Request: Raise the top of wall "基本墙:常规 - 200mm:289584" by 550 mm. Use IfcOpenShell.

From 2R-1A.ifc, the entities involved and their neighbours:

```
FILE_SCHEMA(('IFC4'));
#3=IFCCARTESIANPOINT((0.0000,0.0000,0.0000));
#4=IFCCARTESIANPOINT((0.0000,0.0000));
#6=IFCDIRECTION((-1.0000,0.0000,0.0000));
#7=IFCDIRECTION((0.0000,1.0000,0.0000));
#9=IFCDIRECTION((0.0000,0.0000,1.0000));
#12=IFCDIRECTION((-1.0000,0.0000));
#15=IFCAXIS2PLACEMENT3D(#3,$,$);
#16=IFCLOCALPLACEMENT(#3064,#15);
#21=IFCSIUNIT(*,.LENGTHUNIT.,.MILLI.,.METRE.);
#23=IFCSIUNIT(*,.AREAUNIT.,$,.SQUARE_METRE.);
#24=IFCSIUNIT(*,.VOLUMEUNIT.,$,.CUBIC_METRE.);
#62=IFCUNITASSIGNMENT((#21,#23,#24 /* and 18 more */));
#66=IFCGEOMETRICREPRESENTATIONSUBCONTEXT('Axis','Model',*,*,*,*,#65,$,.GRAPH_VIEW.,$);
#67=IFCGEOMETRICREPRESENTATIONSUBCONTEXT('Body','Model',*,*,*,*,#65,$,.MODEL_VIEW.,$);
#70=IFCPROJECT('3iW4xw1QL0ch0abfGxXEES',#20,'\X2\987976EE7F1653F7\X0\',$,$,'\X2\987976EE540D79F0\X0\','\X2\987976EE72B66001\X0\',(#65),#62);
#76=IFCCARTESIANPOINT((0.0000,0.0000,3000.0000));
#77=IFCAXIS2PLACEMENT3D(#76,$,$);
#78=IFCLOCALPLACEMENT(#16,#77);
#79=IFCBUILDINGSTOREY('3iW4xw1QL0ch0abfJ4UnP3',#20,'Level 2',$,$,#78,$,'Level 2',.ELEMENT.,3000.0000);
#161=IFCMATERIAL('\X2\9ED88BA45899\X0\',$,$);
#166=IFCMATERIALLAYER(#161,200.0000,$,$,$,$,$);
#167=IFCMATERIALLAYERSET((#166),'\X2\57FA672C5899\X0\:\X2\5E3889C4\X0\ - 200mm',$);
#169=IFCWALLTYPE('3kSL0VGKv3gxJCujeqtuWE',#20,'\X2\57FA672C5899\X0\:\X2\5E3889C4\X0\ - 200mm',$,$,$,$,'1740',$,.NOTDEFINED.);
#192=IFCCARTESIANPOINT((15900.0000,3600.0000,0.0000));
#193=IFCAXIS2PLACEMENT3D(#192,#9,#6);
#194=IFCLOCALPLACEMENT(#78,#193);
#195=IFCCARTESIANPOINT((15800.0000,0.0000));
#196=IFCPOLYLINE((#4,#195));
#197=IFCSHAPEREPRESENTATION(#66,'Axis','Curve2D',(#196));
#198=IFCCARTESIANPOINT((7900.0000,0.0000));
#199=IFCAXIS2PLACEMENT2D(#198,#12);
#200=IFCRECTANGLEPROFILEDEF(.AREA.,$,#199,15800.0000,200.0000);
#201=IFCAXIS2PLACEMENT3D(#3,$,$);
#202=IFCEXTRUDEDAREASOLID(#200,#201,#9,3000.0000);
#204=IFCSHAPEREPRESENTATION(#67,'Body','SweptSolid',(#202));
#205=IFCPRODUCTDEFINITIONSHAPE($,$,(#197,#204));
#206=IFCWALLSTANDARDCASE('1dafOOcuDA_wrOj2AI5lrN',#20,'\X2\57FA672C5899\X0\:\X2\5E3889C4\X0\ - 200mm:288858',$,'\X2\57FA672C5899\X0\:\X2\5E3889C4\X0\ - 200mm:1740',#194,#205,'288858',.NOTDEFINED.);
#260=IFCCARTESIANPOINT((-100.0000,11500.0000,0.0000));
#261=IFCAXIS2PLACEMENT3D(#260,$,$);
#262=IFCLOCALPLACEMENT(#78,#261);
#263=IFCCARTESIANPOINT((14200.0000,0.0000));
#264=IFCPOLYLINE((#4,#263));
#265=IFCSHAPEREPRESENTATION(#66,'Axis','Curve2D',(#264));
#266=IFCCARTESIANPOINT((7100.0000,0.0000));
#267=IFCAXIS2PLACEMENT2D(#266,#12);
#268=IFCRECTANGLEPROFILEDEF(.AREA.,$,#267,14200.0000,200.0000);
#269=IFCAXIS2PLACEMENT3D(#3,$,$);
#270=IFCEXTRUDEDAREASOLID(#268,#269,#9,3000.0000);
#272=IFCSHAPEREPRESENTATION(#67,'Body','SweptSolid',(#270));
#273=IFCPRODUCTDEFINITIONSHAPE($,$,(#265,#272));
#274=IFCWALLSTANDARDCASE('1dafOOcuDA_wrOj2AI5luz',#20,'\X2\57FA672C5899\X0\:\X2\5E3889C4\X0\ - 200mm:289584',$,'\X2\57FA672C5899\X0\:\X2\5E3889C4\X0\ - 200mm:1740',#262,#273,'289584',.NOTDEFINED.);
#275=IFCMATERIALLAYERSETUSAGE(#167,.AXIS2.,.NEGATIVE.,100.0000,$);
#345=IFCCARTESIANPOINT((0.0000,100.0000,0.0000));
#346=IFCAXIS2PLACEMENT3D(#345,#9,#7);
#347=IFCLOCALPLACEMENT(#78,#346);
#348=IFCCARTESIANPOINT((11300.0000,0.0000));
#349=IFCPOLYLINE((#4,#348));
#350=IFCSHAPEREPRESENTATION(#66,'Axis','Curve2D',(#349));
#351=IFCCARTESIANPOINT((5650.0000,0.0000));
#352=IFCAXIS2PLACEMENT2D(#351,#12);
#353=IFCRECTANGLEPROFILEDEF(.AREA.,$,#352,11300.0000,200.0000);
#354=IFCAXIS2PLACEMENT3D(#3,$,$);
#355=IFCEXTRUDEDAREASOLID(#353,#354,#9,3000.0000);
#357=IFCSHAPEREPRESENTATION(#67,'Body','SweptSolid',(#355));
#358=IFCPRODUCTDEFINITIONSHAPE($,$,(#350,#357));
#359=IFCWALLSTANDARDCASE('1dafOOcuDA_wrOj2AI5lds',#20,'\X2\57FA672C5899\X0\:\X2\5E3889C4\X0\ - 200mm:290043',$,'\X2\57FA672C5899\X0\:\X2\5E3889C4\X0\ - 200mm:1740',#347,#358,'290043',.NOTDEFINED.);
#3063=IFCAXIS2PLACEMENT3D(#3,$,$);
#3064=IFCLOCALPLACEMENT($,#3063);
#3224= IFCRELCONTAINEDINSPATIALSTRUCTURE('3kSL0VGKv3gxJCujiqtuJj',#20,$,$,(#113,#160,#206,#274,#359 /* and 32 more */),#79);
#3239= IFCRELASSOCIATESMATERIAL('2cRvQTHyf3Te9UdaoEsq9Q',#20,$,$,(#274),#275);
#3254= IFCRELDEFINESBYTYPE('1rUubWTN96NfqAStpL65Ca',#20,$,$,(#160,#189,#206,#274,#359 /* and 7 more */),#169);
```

```python
import ifcopenshell
import ifcopenshell.geom
import ifcopenshell.util.representation
import ifcopenshell.util.shape
import ifcopenshell.util.unit

model = ifcopenshell.open("2R-1A.ifc")
unit_scale = ifcopenshell.util.unit.calculate_unit_scale(model)
settings = ifcopenshell.geom.settings()


def volume(element):
    """Net volume in cubic metres, openings subtracted."""
    shape = ifcopenshell.geom.create_shape(settings, element)
    return ifcopenshell.util.shape.get_volume(shape.geometry)


wall = model.by_guid("1dafOOcuDA_wrOj2AI5luz")
before = volume(wall)

body = ifcopenshell.util.representation.get_representation(wall, "Model", "Body")
solid = body.Items[0]
old_height = solid.Depth
solid.Depth += 0.55 / unit_scale
after = volume(wall)

print(f"height {old_height:g} -> {solid.Depth:g}, volume {before:.3f} -> {after:.3f} m3")

model.write("2R-1A_v2.ifc")
```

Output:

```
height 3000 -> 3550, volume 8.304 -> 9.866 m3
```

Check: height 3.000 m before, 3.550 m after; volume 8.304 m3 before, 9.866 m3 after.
